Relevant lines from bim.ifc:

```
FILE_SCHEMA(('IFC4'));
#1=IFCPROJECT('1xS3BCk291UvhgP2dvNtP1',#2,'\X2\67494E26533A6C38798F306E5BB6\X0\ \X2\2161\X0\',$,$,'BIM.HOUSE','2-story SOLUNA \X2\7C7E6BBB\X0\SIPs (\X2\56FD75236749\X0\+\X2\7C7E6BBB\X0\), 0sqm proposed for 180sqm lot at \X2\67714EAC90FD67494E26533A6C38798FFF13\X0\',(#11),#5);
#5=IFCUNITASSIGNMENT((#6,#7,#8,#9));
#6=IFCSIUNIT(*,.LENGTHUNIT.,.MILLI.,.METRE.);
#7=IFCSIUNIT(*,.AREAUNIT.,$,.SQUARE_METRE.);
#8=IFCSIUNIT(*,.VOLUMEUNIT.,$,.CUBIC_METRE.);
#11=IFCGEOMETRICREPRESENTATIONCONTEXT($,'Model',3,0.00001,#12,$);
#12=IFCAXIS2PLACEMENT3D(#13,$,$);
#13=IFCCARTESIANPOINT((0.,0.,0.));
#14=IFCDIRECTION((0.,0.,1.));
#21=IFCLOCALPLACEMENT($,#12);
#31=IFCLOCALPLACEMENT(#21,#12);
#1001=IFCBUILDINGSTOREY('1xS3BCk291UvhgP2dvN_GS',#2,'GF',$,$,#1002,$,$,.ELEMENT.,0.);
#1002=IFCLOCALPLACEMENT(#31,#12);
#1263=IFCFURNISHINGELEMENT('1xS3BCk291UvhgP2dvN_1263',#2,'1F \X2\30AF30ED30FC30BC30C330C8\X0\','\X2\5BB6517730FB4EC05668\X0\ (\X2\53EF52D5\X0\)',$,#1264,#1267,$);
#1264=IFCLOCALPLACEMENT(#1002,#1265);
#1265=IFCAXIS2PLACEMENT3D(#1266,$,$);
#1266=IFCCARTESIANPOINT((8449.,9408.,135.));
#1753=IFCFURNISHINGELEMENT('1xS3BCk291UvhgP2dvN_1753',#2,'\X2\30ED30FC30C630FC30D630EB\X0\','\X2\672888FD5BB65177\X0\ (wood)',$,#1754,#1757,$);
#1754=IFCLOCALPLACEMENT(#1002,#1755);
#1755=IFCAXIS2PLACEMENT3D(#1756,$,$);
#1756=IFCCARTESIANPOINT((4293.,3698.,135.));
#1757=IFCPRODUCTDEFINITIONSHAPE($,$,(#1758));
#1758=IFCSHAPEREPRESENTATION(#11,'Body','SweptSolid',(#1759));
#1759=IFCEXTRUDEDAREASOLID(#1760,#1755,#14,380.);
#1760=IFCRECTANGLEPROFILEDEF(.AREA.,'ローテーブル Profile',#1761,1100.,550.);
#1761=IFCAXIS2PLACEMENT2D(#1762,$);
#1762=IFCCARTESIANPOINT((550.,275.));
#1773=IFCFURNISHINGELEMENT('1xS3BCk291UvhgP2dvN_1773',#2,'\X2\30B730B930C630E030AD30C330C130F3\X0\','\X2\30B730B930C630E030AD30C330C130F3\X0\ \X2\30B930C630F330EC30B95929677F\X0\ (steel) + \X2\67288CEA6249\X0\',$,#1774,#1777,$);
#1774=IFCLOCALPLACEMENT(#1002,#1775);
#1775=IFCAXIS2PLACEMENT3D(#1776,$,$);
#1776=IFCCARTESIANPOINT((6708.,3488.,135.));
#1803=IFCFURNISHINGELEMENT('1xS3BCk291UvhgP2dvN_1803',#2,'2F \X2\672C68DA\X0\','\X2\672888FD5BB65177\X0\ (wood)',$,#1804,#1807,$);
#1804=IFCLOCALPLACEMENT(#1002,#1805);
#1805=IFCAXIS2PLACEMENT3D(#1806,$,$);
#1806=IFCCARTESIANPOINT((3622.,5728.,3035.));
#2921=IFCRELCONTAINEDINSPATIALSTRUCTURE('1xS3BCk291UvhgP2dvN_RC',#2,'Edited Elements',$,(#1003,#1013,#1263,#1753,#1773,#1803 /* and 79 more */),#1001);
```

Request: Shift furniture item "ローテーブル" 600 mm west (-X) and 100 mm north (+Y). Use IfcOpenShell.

```python
import ifcopenshell
import ifcopenshell.api.geometry
import ifcopenshell.util.placement
import ifcopenshell.util.unit

model = ifcopenshell.open("bim.ifc")
unit_scale = ifcopenshell.util.unit.calculate_unit_scale(model)

item = model.by_id(1753)
matrix = ifcopenshell.util.placement.get_local_placement(item.ObjectPlacement)
matrix[0, 3] -= 0.6 / unit_scale
matrix[1, 3] += 0.1 / unit_scale
ifcopenshell.api.geometry.edit_object_placement(model, product=item, matrix=matrix, is_si=False)

print(ifcopenshell.util.placement.get_local_placement(item.ObjectPlacement).round(3) + 0.0)

model.write("bim_rev.ifc")
```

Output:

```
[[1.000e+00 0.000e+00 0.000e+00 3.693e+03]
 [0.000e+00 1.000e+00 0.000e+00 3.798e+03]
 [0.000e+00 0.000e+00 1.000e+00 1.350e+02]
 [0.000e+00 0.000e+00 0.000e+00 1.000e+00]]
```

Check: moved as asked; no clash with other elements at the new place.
